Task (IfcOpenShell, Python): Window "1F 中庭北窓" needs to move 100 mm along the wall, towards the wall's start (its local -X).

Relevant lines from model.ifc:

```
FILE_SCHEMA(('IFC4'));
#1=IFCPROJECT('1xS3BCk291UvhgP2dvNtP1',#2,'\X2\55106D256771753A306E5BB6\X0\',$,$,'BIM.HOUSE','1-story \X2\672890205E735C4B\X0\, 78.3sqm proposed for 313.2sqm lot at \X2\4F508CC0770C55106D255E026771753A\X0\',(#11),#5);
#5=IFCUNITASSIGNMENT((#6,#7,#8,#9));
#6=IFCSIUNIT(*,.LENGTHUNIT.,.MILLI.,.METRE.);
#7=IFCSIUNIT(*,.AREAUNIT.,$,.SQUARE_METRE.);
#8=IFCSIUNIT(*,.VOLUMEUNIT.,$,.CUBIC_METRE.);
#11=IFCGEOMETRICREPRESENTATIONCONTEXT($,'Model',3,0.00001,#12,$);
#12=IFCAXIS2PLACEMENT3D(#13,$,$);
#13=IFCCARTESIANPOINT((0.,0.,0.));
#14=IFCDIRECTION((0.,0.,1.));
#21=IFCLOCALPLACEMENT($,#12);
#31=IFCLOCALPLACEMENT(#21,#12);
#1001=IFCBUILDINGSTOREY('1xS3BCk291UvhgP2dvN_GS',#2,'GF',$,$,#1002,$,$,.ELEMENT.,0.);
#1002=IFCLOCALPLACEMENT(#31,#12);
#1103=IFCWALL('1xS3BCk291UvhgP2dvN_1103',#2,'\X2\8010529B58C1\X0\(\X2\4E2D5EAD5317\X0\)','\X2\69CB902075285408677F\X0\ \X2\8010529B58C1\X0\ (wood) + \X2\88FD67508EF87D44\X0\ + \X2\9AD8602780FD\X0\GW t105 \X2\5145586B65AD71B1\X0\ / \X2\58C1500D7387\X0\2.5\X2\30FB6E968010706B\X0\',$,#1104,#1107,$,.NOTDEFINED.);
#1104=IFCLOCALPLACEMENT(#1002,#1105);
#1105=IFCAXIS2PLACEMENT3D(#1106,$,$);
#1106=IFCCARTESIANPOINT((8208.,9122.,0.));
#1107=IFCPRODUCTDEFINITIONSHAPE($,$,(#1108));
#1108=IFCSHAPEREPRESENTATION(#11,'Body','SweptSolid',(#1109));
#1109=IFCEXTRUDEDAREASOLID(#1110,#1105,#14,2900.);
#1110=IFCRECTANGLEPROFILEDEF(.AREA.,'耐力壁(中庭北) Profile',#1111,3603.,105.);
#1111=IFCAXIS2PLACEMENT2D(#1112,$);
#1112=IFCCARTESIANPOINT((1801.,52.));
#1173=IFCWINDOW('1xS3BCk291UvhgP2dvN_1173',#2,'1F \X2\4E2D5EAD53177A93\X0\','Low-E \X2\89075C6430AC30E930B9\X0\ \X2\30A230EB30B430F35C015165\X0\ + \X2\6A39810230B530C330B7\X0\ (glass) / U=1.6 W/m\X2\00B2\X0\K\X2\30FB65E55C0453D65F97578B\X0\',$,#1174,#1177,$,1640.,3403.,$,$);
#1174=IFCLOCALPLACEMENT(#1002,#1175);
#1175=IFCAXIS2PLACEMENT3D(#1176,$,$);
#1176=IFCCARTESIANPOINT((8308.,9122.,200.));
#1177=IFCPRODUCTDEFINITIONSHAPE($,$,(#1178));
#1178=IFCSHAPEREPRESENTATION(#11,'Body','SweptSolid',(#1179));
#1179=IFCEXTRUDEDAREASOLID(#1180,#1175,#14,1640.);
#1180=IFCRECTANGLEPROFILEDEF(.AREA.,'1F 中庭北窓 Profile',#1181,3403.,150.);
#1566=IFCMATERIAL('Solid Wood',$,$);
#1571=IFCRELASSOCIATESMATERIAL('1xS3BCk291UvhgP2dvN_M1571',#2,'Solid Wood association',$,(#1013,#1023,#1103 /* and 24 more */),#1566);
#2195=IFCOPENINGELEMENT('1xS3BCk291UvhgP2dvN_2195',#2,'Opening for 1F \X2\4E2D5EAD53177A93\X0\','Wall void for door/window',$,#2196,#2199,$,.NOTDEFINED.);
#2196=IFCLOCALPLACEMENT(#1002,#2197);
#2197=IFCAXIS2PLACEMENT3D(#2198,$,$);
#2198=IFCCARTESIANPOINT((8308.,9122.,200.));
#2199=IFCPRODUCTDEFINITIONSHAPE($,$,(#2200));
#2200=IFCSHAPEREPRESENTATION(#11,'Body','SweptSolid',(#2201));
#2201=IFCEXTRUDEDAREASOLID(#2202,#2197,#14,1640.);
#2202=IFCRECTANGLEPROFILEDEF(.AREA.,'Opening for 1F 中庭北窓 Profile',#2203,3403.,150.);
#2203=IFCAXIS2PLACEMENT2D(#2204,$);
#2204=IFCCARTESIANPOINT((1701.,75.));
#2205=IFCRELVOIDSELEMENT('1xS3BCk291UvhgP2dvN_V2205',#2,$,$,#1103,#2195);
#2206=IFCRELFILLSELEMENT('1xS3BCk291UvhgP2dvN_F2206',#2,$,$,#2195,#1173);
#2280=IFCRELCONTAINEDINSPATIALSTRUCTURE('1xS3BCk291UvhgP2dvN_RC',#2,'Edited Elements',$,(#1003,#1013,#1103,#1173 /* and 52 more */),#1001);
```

```python
import ifcopenshell
import ifcopenshell.api.geometry
import ifcopenshell.util.placement

model = ifcopenshell.open("model.ifc")

window = model.by_guid("1xS3BCk291UvhgP2dvN_1173")
opening = window.FillsVoids[0].RelatingOpeningElement
wall = opening.VoidsElements[0].RelatingBuildingElement

wall_matrix = ifcopenshell.util.placement.get_local_placement(wall.ObjectPlacement)
shift = wall_matrix[:3, 0] * -100.0
before = ifcopenshell.util.placement.get_local_placement(window.ObjectPlacement)[:3, 3].copy()

# The window is not placed relative to its opening, so move both.
for product in (opening, window):
    matrix = ifcopenshell.util.placement.get_local_placement(product.ObjectPlacement)
    matrix[:3, 3] += shift
    ifcopenshell.api.geometry.edit_object_placement(model, product=product, matrix=matrix, is_si=False)

after = ifcopenshell.util.placement.get_local_placement(window.ObjectPlacement)[:3, 3]
print("window moved by", (after - before).round(3) + 0.0)

model.write("model-out.ifc")
```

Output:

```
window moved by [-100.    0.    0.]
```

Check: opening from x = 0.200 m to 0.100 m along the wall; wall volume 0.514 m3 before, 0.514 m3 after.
